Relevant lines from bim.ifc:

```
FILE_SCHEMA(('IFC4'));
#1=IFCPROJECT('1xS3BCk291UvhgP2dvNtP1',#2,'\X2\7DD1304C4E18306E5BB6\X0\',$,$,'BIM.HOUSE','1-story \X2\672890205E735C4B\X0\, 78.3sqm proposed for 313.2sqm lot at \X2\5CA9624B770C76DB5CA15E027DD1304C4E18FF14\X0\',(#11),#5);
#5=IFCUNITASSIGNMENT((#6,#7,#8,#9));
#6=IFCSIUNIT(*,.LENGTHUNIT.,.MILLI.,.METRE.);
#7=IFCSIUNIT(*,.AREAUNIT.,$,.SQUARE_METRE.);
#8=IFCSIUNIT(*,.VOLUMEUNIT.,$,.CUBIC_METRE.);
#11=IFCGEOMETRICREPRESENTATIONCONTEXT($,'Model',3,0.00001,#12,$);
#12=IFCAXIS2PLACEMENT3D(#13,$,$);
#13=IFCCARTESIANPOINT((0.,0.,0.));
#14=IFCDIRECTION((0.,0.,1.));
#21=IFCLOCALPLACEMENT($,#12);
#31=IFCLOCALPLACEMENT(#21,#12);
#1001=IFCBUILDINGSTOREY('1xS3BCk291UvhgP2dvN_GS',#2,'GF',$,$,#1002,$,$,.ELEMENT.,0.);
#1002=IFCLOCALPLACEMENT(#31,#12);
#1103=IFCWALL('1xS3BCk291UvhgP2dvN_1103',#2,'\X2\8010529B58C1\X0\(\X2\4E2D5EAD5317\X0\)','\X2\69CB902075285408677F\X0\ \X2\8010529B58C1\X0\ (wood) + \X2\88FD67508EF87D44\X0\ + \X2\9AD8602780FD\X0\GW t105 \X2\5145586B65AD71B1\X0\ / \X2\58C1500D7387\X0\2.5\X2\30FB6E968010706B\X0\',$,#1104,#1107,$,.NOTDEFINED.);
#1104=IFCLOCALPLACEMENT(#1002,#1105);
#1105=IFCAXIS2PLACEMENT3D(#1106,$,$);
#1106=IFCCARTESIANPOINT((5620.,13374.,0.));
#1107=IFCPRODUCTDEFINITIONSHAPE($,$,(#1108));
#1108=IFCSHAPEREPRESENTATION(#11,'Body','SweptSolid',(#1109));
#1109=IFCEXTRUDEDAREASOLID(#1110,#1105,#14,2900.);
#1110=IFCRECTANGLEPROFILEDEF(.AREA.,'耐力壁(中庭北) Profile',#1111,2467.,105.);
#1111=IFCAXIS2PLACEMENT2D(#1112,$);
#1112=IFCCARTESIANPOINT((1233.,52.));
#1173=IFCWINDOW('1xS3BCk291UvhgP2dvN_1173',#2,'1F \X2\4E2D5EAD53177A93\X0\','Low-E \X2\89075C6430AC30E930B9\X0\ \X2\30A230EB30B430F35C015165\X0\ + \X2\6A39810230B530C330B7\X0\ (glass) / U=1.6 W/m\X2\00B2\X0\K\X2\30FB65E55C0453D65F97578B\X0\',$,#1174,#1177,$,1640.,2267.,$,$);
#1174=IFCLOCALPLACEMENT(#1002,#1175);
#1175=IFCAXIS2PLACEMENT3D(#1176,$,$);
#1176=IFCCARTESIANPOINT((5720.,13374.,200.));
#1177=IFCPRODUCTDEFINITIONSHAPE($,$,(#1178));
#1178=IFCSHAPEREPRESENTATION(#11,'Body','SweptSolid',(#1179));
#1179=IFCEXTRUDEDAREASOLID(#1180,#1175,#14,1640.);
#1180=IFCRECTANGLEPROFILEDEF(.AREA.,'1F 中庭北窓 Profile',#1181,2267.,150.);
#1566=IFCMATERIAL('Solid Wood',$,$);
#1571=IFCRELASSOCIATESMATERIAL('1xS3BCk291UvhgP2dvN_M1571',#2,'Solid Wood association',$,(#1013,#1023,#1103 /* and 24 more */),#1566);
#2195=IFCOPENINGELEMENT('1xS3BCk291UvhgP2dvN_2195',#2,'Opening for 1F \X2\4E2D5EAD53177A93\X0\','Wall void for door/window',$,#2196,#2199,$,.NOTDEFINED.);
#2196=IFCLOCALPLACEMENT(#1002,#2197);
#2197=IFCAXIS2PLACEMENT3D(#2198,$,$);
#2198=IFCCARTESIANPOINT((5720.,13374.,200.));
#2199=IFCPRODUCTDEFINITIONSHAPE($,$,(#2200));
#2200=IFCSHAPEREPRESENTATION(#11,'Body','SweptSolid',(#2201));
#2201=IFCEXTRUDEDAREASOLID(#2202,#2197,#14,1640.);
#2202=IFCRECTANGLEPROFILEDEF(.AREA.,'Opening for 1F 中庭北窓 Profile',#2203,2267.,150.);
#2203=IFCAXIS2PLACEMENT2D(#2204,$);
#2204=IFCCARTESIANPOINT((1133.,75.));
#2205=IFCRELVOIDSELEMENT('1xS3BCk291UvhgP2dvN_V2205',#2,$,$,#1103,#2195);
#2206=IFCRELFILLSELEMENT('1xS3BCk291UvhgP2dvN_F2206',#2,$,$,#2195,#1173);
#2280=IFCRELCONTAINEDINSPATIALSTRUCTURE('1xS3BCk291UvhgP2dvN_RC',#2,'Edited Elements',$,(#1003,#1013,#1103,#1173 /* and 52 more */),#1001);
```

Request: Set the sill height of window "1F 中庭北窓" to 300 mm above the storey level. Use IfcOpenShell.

```python
import numpy as np
import ifcopenshell
import ifcopenshell.api.geometry
import ifcopenshell.geom
import ifcopenshell.util.element
import ifcopenshell.util.placement
import ifcopenshell.util.shape
import ifcopenshell.util.unit

model = ifcopenshell.open("bim.ifc")
unit_scale = ifcopenshell.util.unit.calculate_unit_scale(model)

window = model.by_id(1173)
opening = window.FillsVoids[0].RelatingOpeningElement
storey = ifcopenshell.util.element.get_container(window, ifc_class="IfcBuildingStorey")
level = ifcopenshell.util.placement.get_local_placement(storey.ObjectPlacement)[2, 3]

# The opening's origin need not be at the sill, so measure its lowest point.
shape = ifcopenshell.geom.create_shape(ifcopenshell.geom.settings(), opening)
bottom = ifcopenshell.util.shape.get_shape_bottom_elevation(shape, shape.geometry) / unit_scale
dz = level + 0.3 / unit_scale - bottom

shift = np.array([0.0, 0.0, dz])
# The window is not placed relative to its opening, so move both.
for product in (opening, window):
    matrix = ifcopenshell.util.placement.get_local_placement(product.ObjectPlacement)
    matrix[:3, 3] += shift
    ifcopenshell.api.geometry.edit_object_placement(model, product=product, matrix=matrix, is_si=False)

print(f"moved by {dz * unit_scale:+.3f} m")

model.write("bim-out.ifc")
```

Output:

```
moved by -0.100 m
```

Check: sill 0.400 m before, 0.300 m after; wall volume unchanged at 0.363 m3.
